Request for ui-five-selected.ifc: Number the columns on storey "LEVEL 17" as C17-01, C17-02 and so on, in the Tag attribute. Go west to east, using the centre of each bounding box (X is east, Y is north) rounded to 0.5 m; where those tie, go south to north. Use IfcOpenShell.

First a look at what the model holds.

```python
import ifcopenshell
import ifcopenshell.util.element
import ifcopenshell.util.placement

model = ifcopenshell.open("ui-five-selected.ifc")
print(model.schema)
storey = next(s for s in model.by_type("IfcBuildingStorey") if s.Name == "LEVEL 17")
columns = [e for e in ifcopenshell.util.element.get_decomposition(storey) if e.is_a("IfcColumn")]
for e in sorted(columns, key=lambda e: e.id()):
    origin = ifcopenshell.util.placement.get_local_placement(e.ObjectPlacement)[:3, 3]
    print(e.id(), e.Tag, e.Name, origin.round(2) + 0.0, sep=" | ")
```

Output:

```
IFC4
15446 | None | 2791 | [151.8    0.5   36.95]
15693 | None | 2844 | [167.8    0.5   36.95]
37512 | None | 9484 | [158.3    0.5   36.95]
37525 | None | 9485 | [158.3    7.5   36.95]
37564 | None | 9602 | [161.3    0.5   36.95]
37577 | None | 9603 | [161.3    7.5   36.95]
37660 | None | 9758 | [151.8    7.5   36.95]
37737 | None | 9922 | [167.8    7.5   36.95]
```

```python
import ifcopenshell
import ifcopenshell.geom
import ifcopenshell.util.element
import ifcopenshell.util.shape

model = ifcopenshell.open("ui-five-selected.ifc")
settings = ifcopenshell.geom.settings()
settings.set("use-world-coords", True)


def centre(element):
    shape = ifcopenshell.geom.create_shape(settings, element)
    return ifcopenshell.util.shape.get_bbox_centroid(shape.geometry)


storey = next(s for s in model.by_type("IfcBuildingStorey") if s.Name == "LEVEL 17")
columns = [e for e in ifcopenshell.util.element.get_decomposition(storey) if e.is_a("IfcColumn")]

# Insertion points can sit at a corner or the storey origin, so sort by the geometry (in metres).
centres = {e: centre(e) for e in columns}
columns.sort(key=lambda e: (round(centres[e][0] / 0.5), centres[e][1]))

for i, e in enumerate(columns, start=1):
    number = f"C17-{i:02d}"
    e.Tag = number
    print(e.id(), number)

model.write("ui-five-selected-out.ifc")
```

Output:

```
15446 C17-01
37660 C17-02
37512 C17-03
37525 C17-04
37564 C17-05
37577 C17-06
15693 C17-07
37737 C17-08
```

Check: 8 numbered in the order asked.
